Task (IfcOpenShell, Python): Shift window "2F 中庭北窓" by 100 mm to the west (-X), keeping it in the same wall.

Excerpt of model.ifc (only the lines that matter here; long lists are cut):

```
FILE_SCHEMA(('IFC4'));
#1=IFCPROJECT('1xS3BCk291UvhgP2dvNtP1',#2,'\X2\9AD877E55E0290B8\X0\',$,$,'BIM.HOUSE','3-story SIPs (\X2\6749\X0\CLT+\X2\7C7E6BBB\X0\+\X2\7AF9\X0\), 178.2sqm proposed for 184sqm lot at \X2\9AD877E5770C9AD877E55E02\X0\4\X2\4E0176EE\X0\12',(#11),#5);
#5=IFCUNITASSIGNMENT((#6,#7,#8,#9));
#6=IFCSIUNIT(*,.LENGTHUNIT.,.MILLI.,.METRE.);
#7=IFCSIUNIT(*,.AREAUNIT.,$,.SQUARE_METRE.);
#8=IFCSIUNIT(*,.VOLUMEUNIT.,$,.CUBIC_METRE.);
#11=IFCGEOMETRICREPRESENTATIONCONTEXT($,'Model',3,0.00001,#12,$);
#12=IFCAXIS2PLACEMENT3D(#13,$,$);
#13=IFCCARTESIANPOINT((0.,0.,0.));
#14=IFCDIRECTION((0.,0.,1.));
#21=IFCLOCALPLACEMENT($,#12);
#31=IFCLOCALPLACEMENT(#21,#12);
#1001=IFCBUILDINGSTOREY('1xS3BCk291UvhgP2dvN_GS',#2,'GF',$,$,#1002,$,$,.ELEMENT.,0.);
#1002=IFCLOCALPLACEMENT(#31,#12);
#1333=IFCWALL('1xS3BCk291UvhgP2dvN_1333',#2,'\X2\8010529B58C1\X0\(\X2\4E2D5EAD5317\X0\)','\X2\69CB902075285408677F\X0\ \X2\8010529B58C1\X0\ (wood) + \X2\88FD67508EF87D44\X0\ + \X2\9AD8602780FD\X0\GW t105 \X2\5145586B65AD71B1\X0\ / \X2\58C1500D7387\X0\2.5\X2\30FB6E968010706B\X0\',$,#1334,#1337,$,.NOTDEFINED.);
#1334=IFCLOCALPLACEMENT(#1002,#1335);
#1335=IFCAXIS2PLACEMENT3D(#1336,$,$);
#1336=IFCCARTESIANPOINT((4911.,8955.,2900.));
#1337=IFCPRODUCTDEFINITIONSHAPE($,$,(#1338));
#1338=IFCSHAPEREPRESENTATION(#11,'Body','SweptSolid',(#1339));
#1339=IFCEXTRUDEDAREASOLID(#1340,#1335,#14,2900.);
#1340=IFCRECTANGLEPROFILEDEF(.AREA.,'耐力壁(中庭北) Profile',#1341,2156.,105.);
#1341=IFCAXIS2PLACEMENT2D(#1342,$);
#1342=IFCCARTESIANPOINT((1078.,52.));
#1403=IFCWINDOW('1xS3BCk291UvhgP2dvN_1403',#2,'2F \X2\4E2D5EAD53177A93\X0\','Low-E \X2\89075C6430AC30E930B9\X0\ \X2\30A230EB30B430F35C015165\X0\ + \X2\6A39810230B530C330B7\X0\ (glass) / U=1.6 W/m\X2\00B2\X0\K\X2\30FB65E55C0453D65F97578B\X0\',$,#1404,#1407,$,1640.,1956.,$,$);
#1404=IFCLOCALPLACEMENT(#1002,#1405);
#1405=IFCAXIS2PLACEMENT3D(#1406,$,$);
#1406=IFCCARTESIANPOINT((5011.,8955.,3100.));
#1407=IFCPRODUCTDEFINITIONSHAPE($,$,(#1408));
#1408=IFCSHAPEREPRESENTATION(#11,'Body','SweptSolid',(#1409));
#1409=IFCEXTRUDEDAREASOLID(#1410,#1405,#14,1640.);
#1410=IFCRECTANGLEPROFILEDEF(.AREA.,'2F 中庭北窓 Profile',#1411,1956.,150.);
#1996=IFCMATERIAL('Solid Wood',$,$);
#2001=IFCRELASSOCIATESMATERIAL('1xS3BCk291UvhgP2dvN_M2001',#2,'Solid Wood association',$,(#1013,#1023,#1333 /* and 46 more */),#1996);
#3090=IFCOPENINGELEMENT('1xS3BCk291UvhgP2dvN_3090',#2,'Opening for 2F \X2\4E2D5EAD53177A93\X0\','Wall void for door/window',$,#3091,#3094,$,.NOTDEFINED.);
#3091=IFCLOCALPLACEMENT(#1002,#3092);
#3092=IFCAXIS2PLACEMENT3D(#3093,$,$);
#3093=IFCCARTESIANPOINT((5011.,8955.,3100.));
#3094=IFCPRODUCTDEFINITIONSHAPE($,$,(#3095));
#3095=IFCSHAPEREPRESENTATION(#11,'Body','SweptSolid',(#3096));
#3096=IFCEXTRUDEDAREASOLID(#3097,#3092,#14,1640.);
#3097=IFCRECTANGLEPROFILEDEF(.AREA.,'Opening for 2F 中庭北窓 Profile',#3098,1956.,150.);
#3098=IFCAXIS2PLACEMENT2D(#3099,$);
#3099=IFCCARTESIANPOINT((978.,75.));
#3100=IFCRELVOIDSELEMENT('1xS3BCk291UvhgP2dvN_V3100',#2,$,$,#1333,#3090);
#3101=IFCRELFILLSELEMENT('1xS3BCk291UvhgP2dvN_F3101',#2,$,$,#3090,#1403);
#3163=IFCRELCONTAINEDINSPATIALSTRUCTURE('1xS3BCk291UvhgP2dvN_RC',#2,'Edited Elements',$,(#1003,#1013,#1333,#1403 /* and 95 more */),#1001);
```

```python
import ifcopenshell
import ifcopenshell.api.geometry
import ifcopenshell.util.placement
import ifcopenshell.util.unit

model = ifcopenshell.open("model.ifc")
unit_scale = ifcopenshell.util.unit.calculate_unit_scale(model)

window = model.by_guid("1xS3BCk291UvhgP2dvN_1403")
opening = window.FillsVoids[0].RelatingOpeningElement
wall = opening.VoidsElements[0].RelatingBuildingElement

wall_matrix = ifcopenshell.util.placement.get_local_placement(wall.ObjectPlacement)
shift = wall_matrix[:3, 0] * -0.1 / unit_scale
before = ifcopenshell.util.placement.get_local_placement(window.ObjectPlacement)[:3, 3].copy()

# The window is not placed relative to its opening, so move both.
for product in (opening, window):
    matrix = ifcopenshell.util.placement.get_local_placement(product.ObjectPlacement)
    matrix[:3, 3] += shift
    ifcopenshell.api.geometry.edit_object_placement(model, product=product, matrix=matrix, is_si=False)

after = ifcopenshell.util.placement.get_local_placement(window.ObjectPlacement)[:3, 3]
print("window moved by", (after - before).round(3) + 0.0)

model.write("model-out.ifc")
```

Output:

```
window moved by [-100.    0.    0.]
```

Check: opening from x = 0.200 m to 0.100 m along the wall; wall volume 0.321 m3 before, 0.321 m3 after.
